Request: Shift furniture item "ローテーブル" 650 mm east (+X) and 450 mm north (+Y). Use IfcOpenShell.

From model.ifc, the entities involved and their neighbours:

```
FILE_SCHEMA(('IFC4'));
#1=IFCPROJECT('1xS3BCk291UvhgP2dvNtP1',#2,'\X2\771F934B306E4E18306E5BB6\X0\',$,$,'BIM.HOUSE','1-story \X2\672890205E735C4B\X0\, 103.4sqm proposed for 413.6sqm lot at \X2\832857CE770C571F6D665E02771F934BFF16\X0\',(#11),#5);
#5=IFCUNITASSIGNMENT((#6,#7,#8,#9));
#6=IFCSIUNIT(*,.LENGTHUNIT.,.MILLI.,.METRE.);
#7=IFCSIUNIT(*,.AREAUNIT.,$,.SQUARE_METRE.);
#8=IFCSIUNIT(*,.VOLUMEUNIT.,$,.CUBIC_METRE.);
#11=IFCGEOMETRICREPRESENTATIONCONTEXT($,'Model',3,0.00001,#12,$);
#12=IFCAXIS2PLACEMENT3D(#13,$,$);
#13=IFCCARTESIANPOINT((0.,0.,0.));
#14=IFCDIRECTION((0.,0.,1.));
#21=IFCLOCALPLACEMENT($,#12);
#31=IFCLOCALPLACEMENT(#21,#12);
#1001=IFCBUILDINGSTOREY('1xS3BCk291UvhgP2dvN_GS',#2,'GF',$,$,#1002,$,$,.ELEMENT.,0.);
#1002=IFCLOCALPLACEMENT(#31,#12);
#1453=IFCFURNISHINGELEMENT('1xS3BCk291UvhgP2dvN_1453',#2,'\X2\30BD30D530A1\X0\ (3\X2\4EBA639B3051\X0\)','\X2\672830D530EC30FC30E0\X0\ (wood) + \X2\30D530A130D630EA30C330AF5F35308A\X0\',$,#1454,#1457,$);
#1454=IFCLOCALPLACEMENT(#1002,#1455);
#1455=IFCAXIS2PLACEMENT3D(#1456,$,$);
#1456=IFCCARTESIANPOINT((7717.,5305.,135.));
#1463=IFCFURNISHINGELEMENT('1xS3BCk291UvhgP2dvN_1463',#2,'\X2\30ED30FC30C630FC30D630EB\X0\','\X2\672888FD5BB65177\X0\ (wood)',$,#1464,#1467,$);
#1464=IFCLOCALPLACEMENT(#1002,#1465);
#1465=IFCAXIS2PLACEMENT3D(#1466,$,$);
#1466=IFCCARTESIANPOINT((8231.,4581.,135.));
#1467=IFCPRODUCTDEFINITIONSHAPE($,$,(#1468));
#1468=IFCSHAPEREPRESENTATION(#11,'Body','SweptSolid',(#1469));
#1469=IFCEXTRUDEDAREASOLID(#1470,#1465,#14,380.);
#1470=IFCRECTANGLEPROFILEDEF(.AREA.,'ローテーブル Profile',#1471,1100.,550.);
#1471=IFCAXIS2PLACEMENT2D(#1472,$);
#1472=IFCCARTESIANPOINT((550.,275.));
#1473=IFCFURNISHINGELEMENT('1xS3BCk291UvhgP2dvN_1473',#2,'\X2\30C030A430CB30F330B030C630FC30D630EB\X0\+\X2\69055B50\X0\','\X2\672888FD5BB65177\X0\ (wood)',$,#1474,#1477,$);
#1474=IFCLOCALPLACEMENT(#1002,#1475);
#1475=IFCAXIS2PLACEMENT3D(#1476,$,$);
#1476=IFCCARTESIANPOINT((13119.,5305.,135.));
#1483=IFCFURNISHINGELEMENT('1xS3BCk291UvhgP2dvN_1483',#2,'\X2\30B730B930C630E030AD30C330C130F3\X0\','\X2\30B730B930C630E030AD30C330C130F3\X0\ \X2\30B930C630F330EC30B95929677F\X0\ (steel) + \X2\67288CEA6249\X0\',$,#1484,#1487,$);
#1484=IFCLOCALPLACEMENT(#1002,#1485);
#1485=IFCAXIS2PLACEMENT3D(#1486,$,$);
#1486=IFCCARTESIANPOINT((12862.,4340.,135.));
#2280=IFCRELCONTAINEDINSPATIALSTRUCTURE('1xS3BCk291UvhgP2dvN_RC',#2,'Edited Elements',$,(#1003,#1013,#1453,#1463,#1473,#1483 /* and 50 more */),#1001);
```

```python
import ifcopenshell
import ifcopenshell.api.geometry
import ifcopenshell.util.placement

model = ifcopenshell.open("model.ifc")

item = model.by_guid("1xS3BCk291UvhgP2dvN_1463")
matrix = ifcopenshell.util.placement.get_local_placement(item.ObjectPlacement)
matrix[0, 3] += 650.0
matrix[1, 3] += 450.0
ifcopenshell.api.geometry.edit_object_placement(model, product=item, matrix=matrix, is_si=False)

print(ifcopenshell.util.placement.get_local_placement(item.ObjectPlacement).round(3) + 0.0)

model.write("model_edited.ifc")
```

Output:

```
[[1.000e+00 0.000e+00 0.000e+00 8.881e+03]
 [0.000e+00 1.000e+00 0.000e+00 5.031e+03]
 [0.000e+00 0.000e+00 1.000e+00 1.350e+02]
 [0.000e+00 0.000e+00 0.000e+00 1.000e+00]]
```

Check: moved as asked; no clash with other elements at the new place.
